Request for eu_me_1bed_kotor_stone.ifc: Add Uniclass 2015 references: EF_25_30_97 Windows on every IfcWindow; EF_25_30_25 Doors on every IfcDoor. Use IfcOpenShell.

First a look at what the model holds.

```python
import ifcopenshell

model = ifcopenshell.open("eu_me_1bed_kotor_stone.ifc")
print(model.schema)
print("classifications:", [c.Name for c in model.by_type("IfcClassification")])
for ifc_class in ("IfcDoor", "IfcRoof", "IfcStair", "IfcWall", "IfcWindow"):
    print(ifc_class, len(model.by_type(ifc_class)))
```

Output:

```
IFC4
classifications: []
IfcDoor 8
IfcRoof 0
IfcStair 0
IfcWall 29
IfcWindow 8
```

```python
import ifcopenshell
import ifcopenshell.api.classification

model = ifcopenshell.open("eu_me_1bed_kotor_stone.ifc")

system = ifcopenshell.api.classification.add_classification(model, classification="Uniclass 2015")

codes = {
    "IfcWindow": ("EF_25_30_97", "Windows"),
    "IfcDoor": ("EF_25_30_25", "Doors"),
}
for ifc_class, (code, name) in codes.items():
    products = model.by_type(ifc_class)
    ifcopenshell.api.classification.add_reference(
        model, products=products, classification=system, identification=code, name=name
    )
    print(code, len(products))

model.write("eu_me_1bed_kotor_stone_edited.ifc")
```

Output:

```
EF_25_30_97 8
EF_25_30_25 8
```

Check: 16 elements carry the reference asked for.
